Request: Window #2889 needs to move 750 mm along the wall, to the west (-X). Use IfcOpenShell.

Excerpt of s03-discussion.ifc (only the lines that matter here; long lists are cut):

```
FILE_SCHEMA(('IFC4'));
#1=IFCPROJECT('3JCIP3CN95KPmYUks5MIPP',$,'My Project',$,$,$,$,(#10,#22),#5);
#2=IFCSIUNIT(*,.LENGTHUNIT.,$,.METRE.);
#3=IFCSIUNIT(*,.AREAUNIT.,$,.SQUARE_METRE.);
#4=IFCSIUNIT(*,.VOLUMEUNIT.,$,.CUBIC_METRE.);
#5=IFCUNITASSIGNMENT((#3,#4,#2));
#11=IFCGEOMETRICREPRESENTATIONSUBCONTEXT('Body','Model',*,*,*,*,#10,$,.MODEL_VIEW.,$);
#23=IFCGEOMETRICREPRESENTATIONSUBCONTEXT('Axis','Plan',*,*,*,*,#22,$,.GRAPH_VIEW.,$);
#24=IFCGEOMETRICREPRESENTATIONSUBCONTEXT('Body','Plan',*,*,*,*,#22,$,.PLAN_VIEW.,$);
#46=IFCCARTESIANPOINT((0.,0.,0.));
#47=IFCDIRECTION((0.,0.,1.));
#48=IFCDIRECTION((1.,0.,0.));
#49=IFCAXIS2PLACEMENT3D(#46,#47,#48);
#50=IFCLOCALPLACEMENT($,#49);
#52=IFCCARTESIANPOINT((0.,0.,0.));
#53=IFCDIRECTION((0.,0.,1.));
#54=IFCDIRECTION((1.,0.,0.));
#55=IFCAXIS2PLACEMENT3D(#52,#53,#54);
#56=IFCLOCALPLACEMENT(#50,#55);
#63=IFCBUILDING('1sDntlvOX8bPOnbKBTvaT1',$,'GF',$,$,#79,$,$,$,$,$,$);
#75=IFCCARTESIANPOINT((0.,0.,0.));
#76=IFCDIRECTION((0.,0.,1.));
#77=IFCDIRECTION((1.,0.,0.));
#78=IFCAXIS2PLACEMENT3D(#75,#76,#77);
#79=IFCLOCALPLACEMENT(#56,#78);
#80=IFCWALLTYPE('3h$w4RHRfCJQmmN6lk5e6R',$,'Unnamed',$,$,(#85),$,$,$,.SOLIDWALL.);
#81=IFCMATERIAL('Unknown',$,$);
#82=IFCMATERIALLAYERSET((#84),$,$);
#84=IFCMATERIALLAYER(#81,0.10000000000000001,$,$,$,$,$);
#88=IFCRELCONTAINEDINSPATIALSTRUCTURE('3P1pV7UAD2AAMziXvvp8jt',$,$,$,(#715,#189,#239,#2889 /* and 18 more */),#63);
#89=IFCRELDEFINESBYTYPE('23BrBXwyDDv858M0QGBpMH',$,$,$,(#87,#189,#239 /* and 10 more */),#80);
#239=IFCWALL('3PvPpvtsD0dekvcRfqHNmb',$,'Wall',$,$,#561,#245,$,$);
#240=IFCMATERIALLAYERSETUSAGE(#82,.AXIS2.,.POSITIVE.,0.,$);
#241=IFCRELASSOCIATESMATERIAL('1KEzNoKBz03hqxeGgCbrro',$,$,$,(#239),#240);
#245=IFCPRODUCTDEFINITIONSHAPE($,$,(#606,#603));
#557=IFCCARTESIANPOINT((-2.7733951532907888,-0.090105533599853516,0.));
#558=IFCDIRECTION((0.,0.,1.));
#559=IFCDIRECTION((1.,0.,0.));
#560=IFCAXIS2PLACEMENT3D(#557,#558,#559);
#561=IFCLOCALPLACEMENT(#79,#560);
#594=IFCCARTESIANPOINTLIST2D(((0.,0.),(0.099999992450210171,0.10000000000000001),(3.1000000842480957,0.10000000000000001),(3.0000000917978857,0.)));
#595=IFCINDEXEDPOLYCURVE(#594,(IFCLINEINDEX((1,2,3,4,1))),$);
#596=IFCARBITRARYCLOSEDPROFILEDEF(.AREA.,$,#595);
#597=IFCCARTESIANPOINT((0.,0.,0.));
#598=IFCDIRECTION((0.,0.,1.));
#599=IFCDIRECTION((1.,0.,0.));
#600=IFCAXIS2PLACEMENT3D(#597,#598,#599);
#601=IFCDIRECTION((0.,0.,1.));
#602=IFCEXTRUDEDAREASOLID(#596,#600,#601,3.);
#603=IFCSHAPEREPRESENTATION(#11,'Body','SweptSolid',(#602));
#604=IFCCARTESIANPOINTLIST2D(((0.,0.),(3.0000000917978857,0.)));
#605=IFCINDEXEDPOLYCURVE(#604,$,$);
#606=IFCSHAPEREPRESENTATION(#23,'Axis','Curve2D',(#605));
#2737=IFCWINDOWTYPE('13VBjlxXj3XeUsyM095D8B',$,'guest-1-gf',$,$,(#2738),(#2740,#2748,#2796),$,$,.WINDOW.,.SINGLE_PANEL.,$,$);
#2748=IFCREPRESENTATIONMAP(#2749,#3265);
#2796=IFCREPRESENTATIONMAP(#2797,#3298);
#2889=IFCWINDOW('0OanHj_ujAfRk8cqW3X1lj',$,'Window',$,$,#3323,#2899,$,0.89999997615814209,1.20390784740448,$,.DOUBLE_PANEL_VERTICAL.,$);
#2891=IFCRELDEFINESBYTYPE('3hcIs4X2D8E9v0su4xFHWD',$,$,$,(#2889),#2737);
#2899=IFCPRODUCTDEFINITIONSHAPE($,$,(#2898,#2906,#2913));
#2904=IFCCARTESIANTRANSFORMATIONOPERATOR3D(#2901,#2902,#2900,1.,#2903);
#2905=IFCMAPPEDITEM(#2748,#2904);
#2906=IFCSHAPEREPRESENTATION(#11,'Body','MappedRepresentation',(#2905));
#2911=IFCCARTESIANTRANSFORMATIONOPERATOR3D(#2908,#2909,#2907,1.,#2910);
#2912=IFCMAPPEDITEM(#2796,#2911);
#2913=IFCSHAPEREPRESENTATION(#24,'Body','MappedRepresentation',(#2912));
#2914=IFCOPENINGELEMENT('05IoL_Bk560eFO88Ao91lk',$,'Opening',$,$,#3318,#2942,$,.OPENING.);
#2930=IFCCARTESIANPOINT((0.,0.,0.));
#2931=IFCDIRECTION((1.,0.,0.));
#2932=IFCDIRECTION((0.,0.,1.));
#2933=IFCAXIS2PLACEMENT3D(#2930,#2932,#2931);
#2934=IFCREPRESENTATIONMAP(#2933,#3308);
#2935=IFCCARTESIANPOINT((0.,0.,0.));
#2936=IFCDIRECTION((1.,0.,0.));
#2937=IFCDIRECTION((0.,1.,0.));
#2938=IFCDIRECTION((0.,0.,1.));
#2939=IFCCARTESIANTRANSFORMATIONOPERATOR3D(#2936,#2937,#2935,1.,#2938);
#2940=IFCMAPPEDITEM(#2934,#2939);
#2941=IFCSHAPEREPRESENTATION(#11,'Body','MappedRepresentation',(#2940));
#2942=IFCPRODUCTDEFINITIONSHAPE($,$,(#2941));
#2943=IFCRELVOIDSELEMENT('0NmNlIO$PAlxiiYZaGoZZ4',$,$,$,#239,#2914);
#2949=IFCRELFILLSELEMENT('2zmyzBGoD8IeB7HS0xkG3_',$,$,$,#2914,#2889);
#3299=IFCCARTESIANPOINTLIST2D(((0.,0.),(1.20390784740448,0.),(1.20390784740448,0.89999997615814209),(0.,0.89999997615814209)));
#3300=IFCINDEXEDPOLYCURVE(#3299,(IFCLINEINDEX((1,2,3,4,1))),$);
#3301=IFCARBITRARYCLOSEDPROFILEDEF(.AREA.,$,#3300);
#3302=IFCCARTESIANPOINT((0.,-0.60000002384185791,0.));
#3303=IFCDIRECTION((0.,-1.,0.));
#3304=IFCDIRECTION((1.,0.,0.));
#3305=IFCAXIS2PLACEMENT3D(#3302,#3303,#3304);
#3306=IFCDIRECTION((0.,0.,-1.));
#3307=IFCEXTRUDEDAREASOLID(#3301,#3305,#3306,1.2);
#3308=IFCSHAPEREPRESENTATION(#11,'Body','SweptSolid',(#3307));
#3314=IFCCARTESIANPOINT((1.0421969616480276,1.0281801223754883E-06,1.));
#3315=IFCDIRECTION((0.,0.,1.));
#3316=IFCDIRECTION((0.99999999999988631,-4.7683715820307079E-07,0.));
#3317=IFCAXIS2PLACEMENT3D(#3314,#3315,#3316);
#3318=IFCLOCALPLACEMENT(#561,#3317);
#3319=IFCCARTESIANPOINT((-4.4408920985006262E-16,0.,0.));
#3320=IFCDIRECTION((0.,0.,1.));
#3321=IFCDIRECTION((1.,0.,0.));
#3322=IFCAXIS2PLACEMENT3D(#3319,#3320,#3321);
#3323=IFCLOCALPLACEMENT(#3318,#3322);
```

```python
import ifcopenshell
import ifcopenshell.api.geometry
import ifcopenshell.util.placement
import ifcopenshell.util.unit

model = ifcopenshell.open("s03-discussion.ifc")
unit_scale = ifcopenshell.util.unit.calculate_unit_scale(model)

window = model.by_guid("0OanHj_ujAfRk8cqW3X1lj")
opening = window.FillsVoids[0].RelatingOpeningElement
wall = opening.VoidsElements[0].RelatingBuildingElement

wall_matrix = ifcopenshell.util.placement.get_local_placement(wall.ObjectPlacement)
shift = wall_matrix[:3, 0] * -0.75 / unit_scale
before = ifcopenshell.util.placement.get_local_placement(window.ObjectPlacement)[:3, 3].copy()

# The window is placed relative to its opening, so it follows when the opening moves.
matrix = ifcopenshell.util.placement.get_local_placement(opening.ObjectPlacement)
matrix[:3, 3] += shift
ifcopenshell.api.geometry.edit_object_placement(
    model, product=opening, matrix=matrix, is_si=False, should_transform_children=True
)

after = ifcopenshell.util.placement.get_local_placement(window.ObjectPlacement)[:3, 3]
print("window moved by", (after - before).round(3) + 0.0)

model.write("s03-discussion-out.ifc")
```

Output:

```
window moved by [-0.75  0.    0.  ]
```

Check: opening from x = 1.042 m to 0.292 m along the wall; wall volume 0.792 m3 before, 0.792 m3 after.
